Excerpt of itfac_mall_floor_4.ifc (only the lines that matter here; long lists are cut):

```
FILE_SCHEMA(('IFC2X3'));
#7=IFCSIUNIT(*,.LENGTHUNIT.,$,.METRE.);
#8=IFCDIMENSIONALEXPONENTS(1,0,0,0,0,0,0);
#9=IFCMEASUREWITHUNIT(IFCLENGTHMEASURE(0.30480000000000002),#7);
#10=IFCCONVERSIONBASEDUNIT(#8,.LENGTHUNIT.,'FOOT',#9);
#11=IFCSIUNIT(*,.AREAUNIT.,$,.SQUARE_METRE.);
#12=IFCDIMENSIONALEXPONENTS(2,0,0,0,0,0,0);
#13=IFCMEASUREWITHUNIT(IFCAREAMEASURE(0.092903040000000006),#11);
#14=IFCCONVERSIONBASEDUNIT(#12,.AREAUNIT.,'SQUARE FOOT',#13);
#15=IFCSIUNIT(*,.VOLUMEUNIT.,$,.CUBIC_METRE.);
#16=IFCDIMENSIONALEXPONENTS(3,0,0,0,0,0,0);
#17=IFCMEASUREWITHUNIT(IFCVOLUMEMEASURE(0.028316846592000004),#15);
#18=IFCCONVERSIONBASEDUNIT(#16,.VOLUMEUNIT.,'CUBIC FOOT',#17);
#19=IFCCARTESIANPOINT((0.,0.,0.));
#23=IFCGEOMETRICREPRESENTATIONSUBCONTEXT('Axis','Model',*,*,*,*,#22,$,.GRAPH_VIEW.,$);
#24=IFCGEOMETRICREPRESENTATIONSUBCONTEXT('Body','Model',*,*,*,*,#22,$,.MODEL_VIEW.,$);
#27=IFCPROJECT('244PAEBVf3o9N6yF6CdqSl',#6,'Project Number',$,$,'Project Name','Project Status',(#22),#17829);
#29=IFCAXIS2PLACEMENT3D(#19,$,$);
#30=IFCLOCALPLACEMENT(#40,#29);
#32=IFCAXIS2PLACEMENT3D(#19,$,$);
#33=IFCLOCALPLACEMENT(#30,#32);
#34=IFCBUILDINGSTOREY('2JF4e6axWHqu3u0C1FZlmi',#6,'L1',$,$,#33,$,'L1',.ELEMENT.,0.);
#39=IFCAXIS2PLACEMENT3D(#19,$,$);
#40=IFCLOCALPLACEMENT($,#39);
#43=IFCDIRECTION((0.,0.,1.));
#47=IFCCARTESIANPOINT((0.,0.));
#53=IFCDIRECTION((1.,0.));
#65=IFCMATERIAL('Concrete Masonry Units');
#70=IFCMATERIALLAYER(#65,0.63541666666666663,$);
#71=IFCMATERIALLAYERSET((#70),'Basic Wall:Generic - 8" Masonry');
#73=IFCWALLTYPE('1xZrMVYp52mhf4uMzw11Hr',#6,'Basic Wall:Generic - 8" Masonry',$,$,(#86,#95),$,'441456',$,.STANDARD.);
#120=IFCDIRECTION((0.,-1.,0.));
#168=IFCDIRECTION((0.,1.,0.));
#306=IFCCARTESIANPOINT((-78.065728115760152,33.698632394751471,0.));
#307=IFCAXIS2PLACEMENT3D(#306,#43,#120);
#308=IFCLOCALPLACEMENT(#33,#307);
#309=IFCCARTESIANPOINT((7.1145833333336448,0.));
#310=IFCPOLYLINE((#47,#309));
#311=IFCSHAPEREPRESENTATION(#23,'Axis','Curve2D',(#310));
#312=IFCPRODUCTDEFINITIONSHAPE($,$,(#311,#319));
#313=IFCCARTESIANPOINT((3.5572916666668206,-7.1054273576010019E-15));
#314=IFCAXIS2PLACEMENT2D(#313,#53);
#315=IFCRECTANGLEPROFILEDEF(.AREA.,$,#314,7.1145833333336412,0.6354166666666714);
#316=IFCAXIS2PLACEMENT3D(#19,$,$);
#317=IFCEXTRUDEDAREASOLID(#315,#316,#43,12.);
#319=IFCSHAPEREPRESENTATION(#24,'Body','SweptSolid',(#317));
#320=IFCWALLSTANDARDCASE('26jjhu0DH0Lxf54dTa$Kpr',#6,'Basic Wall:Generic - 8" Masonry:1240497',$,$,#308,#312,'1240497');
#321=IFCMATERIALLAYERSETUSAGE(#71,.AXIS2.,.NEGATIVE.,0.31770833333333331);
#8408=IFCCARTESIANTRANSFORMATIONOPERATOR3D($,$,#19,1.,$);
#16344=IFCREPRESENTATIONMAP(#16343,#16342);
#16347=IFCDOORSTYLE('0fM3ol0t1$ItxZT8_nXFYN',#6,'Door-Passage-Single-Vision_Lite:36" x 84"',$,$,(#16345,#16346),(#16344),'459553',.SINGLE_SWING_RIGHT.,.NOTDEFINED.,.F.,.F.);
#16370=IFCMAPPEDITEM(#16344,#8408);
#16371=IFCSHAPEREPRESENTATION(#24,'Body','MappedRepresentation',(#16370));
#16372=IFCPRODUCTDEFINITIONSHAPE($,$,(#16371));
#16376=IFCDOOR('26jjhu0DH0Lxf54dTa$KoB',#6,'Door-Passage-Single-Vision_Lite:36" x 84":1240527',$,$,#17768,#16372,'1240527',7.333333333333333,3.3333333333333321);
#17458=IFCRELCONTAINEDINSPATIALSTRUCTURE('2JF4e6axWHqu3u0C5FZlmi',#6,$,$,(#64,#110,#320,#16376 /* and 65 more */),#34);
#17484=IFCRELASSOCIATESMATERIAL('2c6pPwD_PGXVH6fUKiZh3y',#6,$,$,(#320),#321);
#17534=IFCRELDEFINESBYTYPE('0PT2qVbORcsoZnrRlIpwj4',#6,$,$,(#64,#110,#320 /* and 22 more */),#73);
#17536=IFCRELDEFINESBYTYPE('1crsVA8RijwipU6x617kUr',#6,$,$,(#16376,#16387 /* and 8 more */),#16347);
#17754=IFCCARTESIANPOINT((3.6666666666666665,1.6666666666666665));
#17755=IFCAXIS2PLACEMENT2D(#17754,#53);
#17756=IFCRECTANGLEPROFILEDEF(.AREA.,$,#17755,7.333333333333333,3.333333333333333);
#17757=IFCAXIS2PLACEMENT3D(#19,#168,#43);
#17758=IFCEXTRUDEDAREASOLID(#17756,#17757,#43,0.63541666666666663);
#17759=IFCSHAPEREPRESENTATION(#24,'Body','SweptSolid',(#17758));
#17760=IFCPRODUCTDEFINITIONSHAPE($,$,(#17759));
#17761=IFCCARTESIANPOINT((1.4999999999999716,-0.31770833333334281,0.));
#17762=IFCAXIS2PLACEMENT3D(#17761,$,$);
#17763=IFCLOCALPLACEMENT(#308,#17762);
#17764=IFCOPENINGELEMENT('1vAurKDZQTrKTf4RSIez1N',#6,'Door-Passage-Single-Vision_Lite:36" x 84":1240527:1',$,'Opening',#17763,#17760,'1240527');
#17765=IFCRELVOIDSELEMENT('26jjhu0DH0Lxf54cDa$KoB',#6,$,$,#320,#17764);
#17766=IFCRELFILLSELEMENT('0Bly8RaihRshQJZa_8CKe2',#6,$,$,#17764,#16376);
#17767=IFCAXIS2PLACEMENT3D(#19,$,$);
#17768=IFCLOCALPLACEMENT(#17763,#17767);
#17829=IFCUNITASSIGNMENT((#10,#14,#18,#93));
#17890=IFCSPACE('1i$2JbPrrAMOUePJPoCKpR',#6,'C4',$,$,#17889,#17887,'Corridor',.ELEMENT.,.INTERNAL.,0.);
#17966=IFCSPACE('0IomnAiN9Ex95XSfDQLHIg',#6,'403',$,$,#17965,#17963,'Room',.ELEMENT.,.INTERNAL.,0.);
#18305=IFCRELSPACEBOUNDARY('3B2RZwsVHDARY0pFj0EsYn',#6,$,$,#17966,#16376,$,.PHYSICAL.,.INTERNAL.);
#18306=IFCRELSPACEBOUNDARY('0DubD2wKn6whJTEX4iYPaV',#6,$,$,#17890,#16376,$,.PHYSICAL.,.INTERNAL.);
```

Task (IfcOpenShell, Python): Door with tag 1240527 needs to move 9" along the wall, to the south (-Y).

```python
import ifcopenshell
import ifcopenshell.api.geometry
import ifcopenshell.util.placement
import ifcopenshell.util.unit

model = ifcopenshell.open("itfac_mall_floor_4.ifc")
unit_scale = ifcopenshell.util.unit.calculate_unit_scale(model)

door = model.by_guid("26jjhu0DH0Lxf54dTa$KoB")
opening = door.FillsVoids[0].RelatingOpeningElement
wall = opening.VoidsElements[0].RelatingBuildingElement

wall_matrix = ifcopenshell.util.placement.get_local_placement(wall.ObjectPlacement)
shift = wall_matrix[:3, 0] * 9 * 0.0254 / unit_scale
before = ifcopenshell.util.placement.get_local_placement(door.ObjectPlacement)[:3, 3].copy()

# The door is placed relative to its opening, so it follows when the opening moves.
matrix = ifcopenshell.util.placement.get_local_placement(opening.ObjectPlacement)
matrix[:3, 3] += shift
ifcopenshell.api.geometry.edit_object_placement(
    model, product=opening, matrix=matrix, is_si=False, should_transform_children=True
)

after = ifcopenshell.util.placement.get_local_placement(door.ObjectPlacement)[:3, 3]
print("door moved by", (after - before).round(3) + 0.0)

model.write("itfac_mall_floor_4_updated.ifc")
```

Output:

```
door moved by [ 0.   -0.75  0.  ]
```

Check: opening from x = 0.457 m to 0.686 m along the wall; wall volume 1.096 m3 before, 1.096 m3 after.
